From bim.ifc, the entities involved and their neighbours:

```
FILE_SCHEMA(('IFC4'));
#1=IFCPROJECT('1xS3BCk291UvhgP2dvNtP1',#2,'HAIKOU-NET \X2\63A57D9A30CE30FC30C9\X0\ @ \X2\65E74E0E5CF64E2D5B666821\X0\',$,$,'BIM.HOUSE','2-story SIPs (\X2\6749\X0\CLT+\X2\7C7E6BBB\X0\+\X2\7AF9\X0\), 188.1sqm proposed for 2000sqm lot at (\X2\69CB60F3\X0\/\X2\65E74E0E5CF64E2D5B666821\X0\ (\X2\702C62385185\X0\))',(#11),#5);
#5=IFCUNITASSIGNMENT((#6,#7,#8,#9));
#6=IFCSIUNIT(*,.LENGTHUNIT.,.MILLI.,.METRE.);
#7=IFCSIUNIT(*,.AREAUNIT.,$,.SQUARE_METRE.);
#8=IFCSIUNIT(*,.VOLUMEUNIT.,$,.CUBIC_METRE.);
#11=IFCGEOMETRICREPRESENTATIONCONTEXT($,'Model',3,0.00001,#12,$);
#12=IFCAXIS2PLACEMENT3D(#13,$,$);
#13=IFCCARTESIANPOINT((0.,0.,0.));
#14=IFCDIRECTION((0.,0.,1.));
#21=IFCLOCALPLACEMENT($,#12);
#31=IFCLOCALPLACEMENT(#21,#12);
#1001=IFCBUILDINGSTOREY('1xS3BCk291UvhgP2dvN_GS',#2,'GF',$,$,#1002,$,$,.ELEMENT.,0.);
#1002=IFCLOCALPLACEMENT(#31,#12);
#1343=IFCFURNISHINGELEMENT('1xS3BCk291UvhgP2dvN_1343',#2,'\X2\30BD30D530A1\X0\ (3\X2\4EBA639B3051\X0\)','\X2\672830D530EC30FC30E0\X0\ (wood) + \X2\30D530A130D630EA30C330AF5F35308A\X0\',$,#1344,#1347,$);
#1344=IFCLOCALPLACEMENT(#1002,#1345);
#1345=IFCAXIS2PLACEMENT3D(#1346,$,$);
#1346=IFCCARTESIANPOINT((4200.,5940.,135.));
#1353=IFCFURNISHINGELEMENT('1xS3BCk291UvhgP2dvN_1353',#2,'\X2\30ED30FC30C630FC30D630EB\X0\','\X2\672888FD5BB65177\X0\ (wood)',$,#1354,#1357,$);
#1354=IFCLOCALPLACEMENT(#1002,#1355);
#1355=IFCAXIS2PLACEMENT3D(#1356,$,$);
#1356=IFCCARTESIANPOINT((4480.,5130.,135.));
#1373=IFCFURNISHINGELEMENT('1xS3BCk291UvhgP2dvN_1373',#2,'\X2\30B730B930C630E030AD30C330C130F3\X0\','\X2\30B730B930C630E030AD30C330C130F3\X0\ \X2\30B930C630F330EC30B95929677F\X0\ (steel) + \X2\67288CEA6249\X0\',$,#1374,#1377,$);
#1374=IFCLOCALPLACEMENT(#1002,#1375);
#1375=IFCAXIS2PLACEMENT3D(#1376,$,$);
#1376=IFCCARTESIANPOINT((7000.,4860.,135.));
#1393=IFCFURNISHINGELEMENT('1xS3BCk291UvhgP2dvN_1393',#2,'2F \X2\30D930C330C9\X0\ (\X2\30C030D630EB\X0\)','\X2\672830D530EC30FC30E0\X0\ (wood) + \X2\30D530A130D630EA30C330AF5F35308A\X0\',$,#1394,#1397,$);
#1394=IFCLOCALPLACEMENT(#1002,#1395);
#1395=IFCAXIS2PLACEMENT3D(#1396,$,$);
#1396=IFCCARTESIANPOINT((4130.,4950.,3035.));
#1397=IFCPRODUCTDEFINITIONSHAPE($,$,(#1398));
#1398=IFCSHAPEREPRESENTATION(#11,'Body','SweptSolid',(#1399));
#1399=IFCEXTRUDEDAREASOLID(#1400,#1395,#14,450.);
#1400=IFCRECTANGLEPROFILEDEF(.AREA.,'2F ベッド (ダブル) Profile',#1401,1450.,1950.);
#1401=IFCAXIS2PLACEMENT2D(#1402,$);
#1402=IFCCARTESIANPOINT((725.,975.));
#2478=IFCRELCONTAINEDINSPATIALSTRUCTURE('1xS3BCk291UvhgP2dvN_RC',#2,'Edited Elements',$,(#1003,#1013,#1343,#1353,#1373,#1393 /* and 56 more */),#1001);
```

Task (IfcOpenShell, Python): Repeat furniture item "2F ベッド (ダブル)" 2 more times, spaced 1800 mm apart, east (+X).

```python
import numpy as np
import ifcopenshell
import ifcopenshell.api.geometry
import ifcopenshell.api.root
import ifcopenshell.util.element
import ifcopenshell.util.placement

model = ifcopenshell.open("bim.ifc")


def reuse_history(source, copy):
    """copy_class also copies each property set's owner history, people and application; keep the originals."""
    for rel in copy.IsDefinedBy:
        if rel.is_a("IfcRelDefinesByProperties") and (history := rel.RelatingPropertyDefinition.OwnerHistory):
            rel.RelatingPropertyDefinition.OwnerHistory = source.OwnerHistory
            ifcopenshell.util.element.remove_deep2(model, history)


source = model.by_id(1393)
base = ifcopenshell.util.placement.get_local_placement(source.ObjectPlacement)
step = np.array([1.0, 0.0, 0.0]) * 1800.0

for i in range(1, 3):
    copy = ifcopenshell.api.root.copy_class(model, product=source)
    copy.Representation = ifcopenshell.util.element.copy_deep(
        model, source.Representation, exclude=["IfcGeometricRepresentationContext", "IfcRepresentationMap"]
    )
    reuse_history(source, copy)
    matrix = base.copy()
    matrix[:3, 3] += i * step
    print("added at", matrix[:3, 3].round(3) + 0.0)
    ifcopenshell.api.geometry.edit_object_placement(model, product=copy, matrix=matrix, is_si=False)

model.write("bim-out.ifc")
```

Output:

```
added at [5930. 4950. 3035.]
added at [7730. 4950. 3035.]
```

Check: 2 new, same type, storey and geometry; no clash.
